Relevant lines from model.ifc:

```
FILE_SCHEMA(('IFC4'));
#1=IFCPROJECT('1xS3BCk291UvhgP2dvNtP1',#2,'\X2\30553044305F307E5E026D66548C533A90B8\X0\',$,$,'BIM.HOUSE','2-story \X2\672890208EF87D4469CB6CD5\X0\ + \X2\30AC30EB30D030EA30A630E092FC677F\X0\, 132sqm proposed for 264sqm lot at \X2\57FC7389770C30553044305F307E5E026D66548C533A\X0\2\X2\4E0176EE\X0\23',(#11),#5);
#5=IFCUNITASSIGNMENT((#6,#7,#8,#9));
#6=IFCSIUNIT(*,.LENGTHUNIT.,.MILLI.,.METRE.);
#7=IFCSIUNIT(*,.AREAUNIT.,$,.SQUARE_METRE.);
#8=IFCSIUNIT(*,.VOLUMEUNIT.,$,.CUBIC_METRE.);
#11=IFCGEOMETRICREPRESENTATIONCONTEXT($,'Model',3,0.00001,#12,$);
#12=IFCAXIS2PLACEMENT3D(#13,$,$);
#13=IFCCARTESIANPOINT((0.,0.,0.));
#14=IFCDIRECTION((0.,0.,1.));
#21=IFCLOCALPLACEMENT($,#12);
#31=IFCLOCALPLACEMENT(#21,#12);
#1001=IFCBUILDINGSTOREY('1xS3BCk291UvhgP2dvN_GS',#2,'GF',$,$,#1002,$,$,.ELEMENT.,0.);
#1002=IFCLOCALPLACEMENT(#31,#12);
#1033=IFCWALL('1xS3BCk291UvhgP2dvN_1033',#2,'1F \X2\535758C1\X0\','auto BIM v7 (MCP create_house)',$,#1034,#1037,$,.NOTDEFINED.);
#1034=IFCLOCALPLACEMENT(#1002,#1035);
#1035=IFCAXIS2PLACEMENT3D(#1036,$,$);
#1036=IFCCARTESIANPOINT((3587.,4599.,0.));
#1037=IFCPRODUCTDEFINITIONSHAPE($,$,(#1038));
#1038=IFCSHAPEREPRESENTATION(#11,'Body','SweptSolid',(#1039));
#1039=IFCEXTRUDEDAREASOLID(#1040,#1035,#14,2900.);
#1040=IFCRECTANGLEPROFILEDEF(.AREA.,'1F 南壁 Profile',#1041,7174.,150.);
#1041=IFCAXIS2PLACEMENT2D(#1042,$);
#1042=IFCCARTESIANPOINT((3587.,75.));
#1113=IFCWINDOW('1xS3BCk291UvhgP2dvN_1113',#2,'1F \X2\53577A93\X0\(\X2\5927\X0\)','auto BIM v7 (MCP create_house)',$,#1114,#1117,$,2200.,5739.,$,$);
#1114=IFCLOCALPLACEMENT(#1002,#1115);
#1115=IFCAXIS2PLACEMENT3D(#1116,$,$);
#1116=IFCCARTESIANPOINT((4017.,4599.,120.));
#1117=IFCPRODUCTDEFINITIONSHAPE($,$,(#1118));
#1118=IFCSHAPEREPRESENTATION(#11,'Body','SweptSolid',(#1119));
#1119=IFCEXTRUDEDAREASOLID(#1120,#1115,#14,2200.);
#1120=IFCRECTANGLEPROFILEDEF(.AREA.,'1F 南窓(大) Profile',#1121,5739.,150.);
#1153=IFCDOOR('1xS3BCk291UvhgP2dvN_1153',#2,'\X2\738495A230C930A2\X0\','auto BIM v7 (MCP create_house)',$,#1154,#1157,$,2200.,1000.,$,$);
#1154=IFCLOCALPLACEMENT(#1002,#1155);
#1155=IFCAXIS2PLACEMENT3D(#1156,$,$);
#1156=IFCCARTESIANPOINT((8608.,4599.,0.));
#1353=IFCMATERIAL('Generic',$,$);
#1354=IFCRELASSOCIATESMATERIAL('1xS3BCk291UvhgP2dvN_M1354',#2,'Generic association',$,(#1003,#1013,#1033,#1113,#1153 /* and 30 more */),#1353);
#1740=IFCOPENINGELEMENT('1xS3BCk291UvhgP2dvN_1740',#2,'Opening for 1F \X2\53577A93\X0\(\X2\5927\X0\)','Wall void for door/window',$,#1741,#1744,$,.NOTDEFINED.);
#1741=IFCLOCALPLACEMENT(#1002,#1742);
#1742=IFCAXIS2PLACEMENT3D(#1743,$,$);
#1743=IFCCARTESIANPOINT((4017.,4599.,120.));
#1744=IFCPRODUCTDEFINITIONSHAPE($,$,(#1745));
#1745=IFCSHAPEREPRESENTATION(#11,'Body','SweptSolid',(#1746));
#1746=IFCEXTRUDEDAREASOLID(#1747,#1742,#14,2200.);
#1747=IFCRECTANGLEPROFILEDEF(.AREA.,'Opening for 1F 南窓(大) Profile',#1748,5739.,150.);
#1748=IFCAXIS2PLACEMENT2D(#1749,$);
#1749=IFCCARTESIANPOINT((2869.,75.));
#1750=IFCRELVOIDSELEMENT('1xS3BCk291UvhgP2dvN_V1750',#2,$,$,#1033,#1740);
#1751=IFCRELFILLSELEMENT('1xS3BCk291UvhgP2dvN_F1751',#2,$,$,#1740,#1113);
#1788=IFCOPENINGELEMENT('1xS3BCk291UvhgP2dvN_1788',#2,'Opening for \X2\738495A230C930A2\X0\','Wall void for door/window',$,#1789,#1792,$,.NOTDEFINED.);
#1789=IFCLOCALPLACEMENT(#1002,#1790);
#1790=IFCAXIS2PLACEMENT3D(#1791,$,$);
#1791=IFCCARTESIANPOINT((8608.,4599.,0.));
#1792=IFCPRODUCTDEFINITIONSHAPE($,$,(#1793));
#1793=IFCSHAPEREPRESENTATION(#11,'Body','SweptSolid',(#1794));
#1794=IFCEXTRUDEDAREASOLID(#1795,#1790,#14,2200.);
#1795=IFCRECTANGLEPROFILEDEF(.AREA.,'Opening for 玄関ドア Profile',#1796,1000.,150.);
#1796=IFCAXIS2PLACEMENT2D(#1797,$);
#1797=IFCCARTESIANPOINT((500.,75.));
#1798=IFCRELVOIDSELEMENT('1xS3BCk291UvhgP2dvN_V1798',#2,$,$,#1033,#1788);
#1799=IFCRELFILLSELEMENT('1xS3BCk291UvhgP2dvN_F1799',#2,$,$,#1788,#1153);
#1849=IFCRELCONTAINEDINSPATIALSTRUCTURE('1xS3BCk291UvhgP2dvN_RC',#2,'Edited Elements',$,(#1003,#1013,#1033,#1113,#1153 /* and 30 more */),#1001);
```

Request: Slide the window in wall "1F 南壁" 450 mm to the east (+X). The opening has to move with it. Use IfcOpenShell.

```python
import ifcopenshell
import ifcopenshell.api.geometry
import ifcopenshell.util.placement

model = ifcopenshell.open("model.ifc")

window = model.by_guid("1xS3BCk291UvhgP2dvN_1113")
opening = window.FillsVoids[0].RelatingOpeningElement
wall = opening.VoidsElements[0].RelatingBuildingElement

wall_matrix = ifcopenshell.util.placement.get_local_placement(wall.ObjectPlacement)
shift = wall_matrix[:3, 0] * 450.0
before = ifcopenshell.util.placement.get_local_placement(window.ObjectPlacement)[:3, 3].copy()

# The window is not placed relative to its opening, so move both.
for product in (opening, window):
    matrix = ifcopenshell.util.placement.get_local_placement(product.ObjectPlacement)
    matrix[:3, 3] += shift
    ifcopenshell.api.geometry.edit_object_placement(model, product=product, matrix=matrix, is_si=False)

after = ifcopenshell.util.placement.get_local_placement(window.ObjectPlacement)[:3, 3]
print("window moved by", (after - before).round(3) + 0.0)

model.write("model_updated.ifc")
```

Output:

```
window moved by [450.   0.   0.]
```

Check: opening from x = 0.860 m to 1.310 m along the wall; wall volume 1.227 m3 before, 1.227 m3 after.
